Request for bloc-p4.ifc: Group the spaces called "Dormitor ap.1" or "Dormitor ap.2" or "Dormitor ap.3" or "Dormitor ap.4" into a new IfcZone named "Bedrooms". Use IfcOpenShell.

First a look at what the model holds.

```python
import ifcopenshell

model = ifcopenshell.open("bloc-p4.ifc")
print(model.schema)
seen = {}
for space in model.by_type("IfcSpace"):
    seen[space.LongName] = seen.get(space.LongName, 0) + 1
for name, count in sorted(seen.items(), key=str):
    print(count, "x", name)
print("zones:", [z.Name for z in model.by_type("IfcZone")][:20])
```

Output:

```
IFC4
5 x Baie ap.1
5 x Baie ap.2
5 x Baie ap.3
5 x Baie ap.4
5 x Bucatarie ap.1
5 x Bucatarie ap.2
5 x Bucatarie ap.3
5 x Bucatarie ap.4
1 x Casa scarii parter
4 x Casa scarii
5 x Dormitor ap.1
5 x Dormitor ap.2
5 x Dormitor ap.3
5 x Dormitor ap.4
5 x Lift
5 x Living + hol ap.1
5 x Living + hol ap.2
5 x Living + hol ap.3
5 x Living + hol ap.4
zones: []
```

```python
import ifcopenshell
import ifcopenshell.api.group
import ifcopenshell.api.root

model = ifcopenshell.open("bloc-p4.ifc")

names = {"Dormitor ap.1", "Dormitor ap.2", "Dormitor ap.3", "Dormitor ap.4"}
spaces = [s for s in model.by_type("IfcSpace") if s.LongName in names]

zone = ifcopenshell.api.root.create_entity(model, ifc_class="IfcZone", name="Bedrooms")
ifcopenshell.api.group.assign_group(model, products=spaces, group=zone)
print(len(spaces), "spaces in", zone.Name)

model.write("bloc-p4_rev.ifc")
```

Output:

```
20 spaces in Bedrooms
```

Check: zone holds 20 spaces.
